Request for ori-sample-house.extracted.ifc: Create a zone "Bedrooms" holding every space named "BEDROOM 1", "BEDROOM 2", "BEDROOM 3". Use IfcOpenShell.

First a look at what the model holds.

```python
import ifcopenshell

model = ifcopenshell.open("ori-sample-house.extracted.ifc")
print(model.schema)
seen = {}
for space in model.by_type("IfcSpace"):
    seen[space.Name] = seen.get(space.Name, 0) + 1
for name, count in sorted(seen.items(), key=str):
    print(count, "x", name)
print("zones:", [z.Name for z in model.by_type("IfcZone")][:20])
```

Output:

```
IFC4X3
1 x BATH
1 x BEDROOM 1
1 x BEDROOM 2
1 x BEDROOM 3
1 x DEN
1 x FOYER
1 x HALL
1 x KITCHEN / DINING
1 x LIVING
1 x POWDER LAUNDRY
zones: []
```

```python
import ifcopenshell
import ifcopenshell.api.group
import ifcopenshell.api.root

model = ifcopenshell.open("ori-sample-house.extracted.ifc")

names = {"BEDROOM 1", "BEDROOM 2", "BEDROOM 3"}
spaces = [s for s in model.by_type("IfcSpace") if s.Name in names]

zone = ifcopenshell.api.root.create_entity(model, ifc_class="IfcZone", name="Bedrooms")
ifcopenshell.api.group.assign_group(model, products=spaces, group=zone)
print(len(spaces), "spaces in", zone.Name)

model.write("ori-sample-house.extracted_edited.ifc")
```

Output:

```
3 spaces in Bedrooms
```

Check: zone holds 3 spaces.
